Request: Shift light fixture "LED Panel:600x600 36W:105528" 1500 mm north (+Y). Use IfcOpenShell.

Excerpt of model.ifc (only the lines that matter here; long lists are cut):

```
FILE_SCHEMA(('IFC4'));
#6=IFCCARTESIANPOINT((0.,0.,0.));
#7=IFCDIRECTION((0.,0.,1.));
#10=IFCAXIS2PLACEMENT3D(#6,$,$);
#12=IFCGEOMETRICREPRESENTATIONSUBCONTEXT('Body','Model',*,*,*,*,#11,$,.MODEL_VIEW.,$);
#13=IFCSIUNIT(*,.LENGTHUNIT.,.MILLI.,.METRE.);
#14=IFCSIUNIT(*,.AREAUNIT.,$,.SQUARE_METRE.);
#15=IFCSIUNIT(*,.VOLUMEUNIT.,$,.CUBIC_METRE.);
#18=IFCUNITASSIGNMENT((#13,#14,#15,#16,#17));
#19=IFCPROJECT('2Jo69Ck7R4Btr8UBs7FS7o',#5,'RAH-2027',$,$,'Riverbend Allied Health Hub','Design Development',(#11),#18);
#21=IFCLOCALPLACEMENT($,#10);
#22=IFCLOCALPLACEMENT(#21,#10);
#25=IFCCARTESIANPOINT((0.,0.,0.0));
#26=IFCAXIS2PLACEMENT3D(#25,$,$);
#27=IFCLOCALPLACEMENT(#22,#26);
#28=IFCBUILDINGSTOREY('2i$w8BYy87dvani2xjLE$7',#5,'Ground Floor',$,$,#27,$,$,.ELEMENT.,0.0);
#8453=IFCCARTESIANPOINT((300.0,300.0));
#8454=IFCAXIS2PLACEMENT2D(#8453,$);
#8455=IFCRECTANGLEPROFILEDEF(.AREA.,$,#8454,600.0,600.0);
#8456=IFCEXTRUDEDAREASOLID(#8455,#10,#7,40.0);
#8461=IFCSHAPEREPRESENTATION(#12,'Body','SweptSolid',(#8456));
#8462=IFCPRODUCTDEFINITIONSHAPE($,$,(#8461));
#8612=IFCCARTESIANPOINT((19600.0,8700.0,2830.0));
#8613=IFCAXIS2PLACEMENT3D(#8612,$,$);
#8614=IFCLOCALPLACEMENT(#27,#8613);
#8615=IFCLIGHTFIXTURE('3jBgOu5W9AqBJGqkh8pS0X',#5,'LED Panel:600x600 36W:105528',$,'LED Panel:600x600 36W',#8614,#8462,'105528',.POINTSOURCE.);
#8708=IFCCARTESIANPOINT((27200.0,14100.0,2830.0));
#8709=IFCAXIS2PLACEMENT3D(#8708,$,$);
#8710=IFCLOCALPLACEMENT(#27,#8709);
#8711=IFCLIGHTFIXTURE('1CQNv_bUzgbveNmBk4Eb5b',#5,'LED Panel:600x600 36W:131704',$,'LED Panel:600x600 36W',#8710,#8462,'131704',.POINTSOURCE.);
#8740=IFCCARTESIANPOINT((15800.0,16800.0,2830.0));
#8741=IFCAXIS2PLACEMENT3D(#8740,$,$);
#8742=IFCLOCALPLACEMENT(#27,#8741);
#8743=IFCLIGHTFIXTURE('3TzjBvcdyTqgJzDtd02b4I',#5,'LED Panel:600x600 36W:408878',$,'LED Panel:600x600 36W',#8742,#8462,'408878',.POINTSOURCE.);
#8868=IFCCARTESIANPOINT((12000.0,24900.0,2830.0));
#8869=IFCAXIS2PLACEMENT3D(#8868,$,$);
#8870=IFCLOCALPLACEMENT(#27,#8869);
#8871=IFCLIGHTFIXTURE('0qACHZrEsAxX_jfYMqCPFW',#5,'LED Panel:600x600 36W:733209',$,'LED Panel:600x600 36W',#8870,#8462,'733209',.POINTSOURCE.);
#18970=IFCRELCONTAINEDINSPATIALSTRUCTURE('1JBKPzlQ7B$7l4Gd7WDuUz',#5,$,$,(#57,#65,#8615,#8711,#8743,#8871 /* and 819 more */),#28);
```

```python
import ifcopenshell
import ifcopenshell.api.geometry
import ifcopenshell.util.placement

model = ifcopenshell.open("model.ifc")

item = model.by_id(8615)
matrix = ifcopenshell.util.placement.get_local_placement(item.ObjectPlacement)
matrix[1, 3] += 1500.0
ifcopenshell.api.geometry.edit_object_placement(model, product=item, matrix=matrix, is_si=False)

print(ifcopenshell.util.placement.get_local_placement(item.ObjectPlacement).round(3) + 0.0)

model.write("model_v2.ifc")
```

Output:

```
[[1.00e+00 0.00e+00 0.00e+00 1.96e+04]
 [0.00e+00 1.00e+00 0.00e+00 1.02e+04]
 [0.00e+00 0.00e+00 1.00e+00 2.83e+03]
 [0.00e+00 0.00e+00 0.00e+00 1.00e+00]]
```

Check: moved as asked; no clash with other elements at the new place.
